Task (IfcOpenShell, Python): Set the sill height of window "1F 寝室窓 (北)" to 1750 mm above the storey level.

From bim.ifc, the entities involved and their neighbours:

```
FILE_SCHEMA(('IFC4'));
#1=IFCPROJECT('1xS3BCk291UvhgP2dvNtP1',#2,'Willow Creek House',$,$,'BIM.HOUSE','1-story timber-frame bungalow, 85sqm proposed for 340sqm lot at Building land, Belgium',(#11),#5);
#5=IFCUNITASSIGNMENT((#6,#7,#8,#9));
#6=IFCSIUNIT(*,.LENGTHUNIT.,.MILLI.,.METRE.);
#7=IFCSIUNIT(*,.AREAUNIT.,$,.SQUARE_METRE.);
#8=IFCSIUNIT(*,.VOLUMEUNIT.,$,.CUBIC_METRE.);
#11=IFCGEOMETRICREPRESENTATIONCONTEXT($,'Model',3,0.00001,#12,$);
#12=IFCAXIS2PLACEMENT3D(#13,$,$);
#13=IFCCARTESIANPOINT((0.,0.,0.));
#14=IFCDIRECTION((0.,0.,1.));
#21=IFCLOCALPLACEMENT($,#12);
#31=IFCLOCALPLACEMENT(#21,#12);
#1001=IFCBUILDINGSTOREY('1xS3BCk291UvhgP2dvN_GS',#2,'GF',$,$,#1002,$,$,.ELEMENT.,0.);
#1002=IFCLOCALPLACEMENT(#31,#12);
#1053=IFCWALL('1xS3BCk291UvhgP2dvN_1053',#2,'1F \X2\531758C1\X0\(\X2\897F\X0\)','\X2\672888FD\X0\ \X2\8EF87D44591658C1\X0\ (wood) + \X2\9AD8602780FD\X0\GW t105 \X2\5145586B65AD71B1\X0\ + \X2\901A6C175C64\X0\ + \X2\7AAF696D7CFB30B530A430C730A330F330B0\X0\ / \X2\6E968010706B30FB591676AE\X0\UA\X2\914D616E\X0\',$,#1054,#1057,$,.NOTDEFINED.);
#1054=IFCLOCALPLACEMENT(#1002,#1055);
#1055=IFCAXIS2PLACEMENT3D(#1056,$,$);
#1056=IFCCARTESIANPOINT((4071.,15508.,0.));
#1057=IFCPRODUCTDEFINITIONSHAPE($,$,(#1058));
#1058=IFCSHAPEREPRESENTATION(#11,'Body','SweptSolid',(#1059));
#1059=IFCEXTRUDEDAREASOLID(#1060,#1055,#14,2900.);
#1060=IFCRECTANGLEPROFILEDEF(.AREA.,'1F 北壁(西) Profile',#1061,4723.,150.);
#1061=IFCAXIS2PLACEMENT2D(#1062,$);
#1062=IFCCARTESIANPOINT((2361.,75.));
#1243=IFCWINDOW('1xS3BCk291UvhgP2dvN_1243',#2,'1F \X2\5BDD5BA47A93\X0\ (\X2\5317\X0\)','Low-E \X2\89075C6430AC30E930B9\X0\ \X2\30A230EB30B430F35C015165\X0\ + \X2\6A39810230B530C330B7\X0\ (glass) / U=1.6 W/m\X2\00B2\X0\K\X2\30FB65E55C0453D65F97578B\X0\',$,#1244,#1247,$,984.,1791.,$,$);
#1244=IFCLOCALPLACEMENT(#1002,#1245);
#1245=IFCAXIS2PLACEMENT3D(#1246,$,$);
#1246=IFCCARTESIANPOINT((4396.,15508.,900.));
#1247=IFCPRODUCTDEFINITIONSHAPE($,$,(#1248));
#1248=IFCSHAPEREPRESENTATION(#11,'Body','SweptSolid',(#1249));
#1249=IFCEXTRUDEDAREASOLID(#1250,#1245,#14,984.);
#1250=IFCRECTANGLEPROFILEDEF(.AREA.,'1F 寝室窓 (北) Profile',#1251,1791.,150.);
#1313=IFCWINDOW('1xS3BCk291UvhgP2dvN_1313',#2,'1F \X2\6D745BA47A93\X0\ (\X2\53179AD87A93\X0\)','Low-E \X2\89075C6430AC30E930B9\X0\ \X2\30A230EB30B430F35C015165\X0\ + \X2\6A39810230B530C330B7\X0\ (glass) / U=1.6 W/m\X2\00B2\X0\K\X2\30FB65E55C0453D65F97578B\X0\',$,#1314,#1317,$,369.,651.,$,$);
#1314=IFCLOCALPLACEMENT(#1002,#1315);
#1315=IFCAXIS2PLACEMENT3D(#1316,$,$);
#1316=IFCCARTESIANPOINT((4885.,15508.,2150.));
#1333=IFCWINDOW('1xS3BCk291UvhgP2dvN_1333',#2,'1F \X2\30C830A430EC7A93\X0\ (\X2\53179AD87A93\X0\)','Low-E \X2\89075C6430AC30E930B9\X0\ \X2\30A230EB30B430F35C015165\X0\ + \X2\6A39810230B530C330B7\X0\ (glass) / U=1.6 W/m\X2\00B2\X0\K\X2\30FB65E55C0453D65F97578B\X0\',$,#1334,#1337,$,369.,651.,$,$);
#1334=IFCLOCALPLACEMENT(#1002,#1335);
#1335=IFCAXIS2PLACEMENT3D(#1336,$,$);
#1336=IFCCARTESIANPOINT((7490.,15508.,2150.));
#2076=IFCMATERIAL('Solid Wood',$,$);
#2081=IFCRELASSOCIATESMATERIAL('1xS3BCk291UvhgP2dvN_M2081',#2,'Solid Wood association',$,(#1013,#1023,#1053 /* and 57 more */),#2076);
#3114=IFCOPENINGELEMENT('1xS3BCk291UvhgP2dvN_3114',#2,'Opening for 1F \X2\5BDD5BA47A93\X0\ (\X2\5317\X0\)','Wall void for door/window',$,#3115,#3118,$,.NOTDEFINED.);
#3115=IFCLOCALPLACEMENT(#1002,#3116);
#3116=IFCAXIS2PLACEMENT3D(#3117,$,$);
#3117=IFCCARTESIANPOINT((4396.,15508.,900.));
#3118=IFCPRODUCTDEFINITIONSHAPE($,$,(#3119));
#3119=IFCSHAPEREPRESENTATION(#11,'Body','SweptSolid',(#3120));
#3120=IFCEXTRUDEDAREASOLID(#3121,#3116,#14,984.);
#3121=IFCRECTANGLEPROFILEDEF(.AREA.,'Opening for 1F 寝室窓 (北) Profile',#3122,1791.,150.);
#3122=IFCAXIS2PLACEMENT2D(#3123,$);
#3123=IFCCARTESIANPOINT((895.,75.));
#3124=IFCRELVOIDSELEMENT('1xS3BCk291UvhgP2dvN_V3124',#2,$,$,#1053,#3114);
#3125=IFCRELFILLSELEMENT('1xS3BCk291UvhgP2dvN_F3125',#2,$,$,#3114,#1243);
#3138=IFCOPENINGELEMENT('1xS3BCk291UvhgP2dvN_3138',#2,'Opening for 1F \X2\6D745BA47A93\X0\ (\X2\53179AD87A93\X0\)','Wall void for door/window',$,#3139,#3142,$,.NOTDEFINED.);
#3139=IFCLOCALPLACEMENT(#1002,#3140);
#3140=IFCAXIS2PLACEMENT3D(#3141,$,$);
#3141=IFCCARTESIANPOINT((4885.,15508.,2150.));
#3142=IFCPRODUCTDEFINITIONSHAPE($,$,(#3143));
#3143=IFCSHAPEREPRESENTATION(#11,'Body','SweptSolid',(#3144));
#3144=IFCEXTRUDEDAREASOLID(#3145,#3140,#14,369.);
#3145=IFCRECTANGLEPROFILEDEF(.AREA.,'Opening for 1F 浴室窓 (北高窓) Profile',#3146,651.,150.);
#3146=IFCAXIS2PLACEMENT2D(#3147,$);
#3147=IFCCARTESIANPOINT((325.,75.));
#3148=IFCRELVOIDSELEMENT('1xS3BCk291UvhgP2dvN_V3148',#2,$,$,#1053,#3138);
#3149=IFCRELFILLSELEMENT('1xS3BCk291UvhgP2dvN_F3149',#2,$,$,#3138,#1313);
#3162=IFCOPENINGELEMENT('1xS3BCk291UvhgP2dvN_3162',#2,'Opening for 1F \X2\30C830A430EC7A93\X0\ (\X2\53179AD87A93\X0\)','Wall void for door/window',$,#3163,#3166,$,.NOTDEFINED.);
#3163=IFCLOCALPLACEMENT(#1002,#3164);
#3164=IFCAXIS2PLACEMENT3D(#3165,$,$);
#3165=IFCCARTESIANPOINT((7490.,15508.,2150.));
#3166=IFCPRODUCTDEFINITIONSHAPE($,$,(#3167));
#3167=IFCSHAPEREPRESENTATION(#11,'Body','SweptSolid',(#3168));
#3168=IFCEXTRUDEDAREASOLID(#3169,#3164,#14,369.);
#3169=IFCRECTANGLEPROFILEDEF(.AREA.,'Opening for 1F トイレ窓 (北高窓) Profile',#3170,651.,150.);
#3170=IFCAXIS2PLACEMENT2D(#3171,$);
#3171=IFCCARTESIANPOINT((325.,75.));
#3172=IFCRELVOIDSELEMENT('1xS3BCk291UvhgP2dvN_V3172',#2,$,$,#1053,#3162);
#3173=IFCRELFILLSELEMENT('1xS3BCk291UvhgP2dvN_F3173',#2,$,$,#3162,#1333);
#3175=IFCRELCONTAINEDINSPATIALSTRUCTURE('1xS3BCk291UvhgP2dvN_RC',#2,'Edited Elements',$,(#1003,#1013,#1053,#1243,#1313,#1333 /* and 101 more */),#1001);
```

```python
import numpy as np
import ifcopenshell
import ifcopenshell.api.geometry
import ifcopenshell.geom
import ifcopenshell.util.element
import ifcopenshell.util.placement
import ifcopenshell.util.shape
import ifcopenshell.util.unit

model = ifcopenshell.open("bim.ifc")
unit_scale = ifcopenshell.util.unit.calculate_unit_scale(model)

window = model.by_guid("1xS3BCk291UvhgP2dvN_1243")
opening = window.FillsVoids[0].RelatingOpeningElement
storey = ifcopenshell.util.element.get_container(window, ifc_class="IfcBuildingStorey")
level = ifcopenshell.util.placement.get_local_placement(storey.ObjectPlacement)[2, 3]

# The opening's origin need not be at the sill, so measure its lowest point.
shape = ifcopenshell.geom.create_shape(ifcopenshell.geom.settings(), opening)
bottom = ifcopenshell.util.shape.get_shape_bottom_elevation(shape, shape.geometry) / unit_scale
dz = level + 1.75 / unit_scale - bottom

shift = np.array([0.0, 0.0, dz])
# The window is not placed relative to its opening, so move both.
for product in (opening, window):
    matrix = ifcopenshell.util.placement.get_local_placement(product.ObjectPlacement)
    matrix[:3, 3] += shift
    ifcopenshell.api.geometry.edit_object_placement(model, product=product, matrix=matrix, is_si=False)

print(f"moved by {dz * unit_scale:+.3f} m")

model.write("bim_rev.ifc")
```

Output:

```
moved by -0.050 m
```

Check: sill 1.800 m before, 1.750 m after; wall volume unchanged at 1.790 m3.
